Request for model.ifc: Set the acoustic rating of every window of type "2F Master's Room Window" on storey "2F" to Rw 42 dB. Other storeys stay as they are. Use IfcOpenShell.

First a look at what the model holds.

```python
import ifcopenshell
import ifcopenshell.util.element

model = ifcopenshell.open("model.ifc")
print(model.schema)
storey = next(s for s in model.by_type("IfcBuildingStorey") if s.Name == "2F")
windows = [e for e in ifcopenshell.util.element.get_decomposition(storey) if e.is_a("IfcWindow")]
seen = {}
for e in windows:
    element_type = ifcopenshell.util.element.get_type(e)
    key = (element_type.Name if element_type != e and element_type else None, ifcopenshell.util.element.get_pset(e, "Pset_WindowCommon", "AcousticRating"))
    seen[key] = seen.get(key, 0) + 1
for (name, value), count in sorted(seen.items(), key=str):
    print(count, "x", name, "|", value)
```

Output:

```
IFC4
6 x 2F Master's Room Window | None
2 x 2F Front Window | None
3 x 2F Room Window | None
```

```python
import ifcopenshell
import ifcopenshell.api.pset
import ifcopenshell.util.element

model = ifcopenshell.open("model.ifc")

storey = next(s for s in model.by_type("IfcBuildingStorey") if s.Name == "2F")
windows = [e for e in ifcopenshell.util.element.get_decomposition(storey) if e.is_a("IfcWindow")]

count = 0
for e in windows:
    element_type = ifcopenshell.util.element.get_type(e)
    if element_type in (None, e) or element_type.Name != "2F Master's Room Window":
        continue
    # add_pset returns the element's existing set when there is one.
    pset = ifcopenshell.api.pset.add_pset(model, product=e, name="Pset_WindowCommon")
    ifcopenshell.api.pset.edit_pset(model, pset=pset, properties={"AcousticRating": "Rw 42 dB"})
    count += 1

print(count, "windows updated")

model.write("model-out.ifc")
```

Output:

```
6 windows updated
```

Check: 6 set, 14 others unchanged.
